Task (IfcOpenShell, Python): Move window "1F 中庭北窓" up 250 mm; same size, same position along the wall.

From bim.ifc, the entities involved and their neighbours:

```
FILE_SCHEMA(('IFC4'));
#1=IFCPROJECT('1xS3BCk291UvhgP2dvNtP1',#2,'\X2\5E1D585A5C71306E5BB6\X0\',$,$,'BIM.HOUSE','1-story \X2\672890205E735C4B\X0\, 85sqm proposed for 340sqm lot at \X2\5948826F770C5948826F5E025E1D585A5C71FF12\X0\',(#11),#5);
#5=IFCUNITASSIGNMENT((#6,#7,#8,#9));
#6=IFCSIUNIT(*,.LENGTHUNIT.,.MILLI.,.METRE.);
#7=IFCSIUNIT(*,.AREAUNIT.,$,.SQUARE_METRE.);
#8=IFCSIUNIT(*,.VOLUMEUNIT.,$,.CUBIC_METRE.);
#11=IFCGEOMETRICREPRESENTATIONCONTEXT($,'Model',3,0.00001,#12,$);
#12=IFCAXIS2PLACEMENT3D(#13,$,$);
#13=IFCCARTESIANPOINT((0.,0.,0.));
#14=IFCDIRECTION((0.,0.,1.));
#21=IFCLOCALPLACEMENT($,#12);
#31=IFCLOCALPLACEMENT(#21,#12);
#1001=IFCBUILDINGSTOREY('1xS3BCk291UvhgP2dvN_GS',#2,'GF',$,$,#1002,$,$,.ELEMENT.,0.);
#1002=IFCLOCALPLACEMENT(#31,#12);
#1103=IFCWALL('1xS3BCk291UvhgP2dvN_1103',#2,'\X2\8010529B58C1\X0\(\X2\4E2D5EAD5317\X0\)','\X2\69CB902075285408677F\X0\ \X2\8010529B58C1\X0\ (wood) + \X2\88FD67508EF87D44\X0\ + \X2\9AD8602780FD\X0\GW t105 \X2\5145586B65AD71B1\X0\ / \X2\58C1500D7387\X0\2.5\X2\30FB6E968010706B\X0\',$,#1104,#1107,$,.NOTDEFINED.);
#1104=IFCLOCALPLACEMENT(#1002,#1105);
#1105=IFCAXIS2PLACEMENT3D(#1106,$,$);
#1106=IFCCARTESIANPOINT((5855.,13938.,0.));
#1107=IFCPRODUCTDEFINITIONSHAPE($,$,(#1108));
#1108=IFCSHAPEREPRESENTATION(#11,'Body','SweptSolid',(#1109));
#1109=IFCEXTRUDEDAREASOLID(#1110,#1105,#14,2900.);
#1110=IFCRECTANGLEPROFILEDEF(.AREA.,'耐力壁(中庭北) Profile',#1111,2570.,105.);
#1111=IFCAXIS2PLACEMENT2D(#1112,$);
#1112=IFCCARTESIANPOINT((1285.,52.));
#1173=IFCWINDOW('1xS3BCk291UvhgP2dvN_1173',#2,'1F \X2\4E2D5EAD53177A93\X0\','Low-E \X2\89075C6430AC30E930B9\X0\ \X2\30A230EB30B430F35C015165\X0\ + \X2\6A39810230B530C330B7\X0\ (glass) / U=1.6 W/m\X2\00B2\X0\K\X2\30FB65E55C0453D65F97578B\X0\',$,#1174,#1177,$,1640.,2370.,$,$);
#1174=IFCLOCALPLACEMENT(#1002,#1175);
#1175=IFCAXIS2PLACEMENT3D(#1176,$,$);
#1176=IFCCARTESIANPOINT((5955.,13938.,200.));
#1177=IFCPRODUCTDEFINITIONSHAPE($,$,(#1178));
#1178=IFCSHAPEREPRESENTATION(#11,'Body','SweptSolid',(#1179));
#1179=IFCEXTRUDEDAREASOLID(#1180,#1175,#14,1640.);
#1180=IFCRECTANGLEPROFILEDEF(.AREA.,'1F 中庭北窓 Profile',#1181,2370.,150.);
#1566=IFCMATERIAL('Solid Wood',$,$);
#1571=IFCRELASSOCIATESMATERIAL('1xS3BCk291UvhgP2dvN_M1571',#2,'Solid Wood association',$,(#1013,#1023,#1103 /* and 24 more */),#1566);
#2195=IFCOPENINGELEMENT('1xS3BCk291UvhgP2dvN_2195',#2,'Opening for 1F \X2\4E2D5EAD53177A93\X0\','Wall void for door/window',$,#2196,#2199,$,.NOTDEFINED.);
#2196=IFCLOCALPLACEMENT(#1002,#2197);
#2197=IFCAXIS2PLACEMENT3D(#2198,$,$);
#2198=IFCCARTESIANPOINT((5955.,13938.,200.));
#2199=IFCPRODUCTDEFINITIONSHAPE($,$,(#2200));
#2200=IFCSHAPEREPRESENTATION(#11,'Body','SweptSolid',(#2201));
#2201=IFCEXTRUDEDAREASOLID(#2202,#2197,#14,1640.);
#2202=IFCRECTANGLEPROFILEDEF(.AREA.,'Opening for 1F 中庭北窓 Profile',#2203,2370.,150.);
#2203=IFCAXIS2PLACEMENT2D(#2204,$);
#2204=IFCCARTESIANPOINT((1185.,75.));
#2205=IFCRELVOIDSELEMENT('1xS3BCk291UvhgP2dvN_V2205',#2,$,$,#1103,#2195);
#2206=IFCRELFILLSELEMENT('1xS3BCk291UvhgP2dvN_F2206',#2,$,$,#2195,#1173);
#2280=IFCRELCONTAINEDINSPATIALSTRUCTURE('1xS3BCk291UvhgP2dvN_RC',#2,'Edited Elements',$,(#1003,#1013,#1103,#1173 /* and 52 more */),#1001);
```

```python
import numpy as np
import ifcopenshell
import ifcopenshell.api.geometry
import ifcopenshell.util.placement
import ifcopenshell.util.unit

model = ifcopenshell.open("bim.ifc")
unit_scale = ifcopenshell.util.unit.calculate_unit_scale(model)

window = model.by_guid("1xS3BCk291UvhgP2dvN_1173")
opening = window.FillsVoids[0].RelatingOpeningElement
dz = 0.25 / unit_scale

shift = np.array([0.0, 0.0, dz])
# The window is not placed relative to its opening, so move both.
for product in (opening, window):
    matrix = ifcopenshell.util.placement.get_local_placement(product.ObjectPlacement)
    matrix[:3, 3] += shift
    ifcopenshell.api.geometry.edit_object_placement(model, product=product, matrix=matrix, is_si=False)

print(f"moved by {dz * unit_scale:+.3f} m")

model.write("bim_v2.ifc")
```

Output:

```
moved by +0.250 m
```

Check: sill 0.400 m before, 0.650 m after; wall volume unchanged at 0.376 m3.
